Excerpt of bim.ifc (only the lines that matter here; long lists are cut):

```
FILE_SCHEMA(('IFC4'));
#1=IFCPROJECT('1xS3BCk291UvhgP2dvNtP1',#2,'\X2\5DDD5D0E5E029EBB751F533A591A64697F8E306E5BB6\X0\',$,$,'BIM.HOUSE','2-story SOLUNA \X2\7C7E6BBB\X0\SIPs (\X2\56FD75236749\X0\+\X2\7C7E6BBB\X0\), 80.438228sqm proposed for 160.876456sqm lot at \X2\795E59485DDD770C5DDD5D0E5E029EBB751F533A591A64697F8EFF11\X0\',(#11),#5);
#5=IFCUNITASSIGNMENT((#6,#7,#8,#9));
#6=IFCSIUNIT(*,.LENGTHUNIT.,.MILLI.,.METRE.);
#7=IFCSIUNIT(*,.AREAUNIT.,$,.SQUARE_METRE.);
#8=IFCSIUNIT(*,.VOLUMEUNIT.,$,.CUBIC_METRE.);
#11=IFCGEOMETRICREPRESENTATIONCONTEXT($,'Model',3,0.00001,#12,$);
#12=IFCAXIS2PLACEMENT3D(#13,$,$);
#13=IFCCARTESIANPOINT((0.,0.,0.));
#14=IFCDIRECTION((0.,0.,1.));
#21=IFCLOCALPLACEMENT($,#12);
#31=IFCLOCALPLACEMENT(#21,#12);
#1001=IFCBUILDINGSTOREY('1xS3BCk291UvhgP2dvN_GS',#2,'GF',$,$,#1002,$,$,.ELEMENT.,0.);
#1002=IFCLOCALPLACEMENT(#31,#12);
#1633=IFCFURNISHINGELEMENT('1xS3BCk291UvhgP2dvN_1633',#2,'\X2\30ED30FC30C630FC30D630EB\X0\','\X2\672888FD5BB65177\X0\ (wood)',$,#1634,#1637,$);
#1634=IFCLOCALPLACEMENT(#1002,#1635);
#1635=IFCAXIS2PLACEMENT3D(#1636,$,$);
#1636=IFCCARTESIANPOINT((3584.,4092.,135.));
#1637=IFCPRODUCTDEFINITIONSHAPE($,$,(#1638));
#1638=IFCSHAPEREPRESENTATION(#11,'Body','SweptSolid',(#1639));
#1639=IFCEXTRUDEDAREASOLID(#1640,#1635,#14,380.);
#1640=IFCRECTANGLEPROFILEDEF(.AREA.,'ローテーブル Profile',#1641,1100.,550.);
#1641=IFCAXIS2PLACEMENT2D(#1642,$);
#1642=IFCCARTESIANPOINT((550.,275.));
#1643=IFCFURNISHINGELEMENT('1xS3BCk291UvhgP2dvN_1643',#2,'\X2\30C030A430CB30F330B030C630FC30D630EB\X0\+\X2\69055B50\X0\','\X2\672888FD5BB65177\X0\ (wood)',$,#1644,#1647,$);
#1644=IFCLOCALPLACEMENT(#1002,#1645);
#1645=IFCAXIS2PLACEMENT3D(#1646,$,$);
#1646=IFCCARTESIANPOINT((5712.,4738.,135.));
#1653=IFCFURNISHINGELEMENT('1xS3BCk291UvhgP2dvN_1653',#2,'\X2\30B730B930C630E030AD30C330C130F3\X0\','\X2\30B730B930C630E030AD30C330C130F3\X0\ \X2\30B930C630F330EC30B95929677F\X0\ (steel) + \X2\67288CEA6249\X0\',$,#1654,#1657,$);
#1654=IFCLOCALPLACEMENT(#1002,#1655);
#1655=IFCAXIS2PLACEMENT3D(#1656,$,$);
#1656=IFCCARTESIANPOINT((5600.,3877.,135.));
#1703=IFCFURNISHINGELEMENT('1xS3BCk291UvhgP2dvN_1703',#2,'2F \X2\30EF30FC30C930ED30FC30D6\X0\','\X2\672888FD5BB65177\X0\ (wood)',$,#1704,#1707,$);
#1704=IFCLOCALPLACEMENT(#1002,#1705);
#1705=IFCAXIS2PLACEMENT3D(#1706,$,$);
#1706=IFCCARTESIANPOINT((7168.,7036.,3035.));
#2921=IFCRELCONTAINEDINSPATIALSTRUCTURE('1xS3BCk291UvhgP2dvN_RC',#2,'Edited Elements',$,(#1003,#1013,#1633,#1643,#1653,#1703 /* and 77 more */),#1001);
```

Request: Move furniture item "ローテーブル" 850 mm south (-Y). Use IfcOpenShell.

```python
import ifcopenshell
import ifcopenshell.api.geometry
import ifcopenshell.util.placement
import ifcopenshell.util.unit

model = ifcopenshell.open("bim.ifc")
unit_scale = ifcopenshell.util.unit.calculate_unit_scale(model)

item = model.by_id(1633)
matrix = ifcopenshell.util.placement.get_local_placement(item.ObjectPlacement)
matrix[1, 3] -= 0.85 / unit_scale
ifcopenshell.api.geometry.edit_object_placement(model, product=item, matrix=matrix, is_si=False)

print(ifcopenshell.util.placement.get_local_placement(item.ObjectPlacement).round(3) + 0.0)

model.write("bim_updated.ifc")
```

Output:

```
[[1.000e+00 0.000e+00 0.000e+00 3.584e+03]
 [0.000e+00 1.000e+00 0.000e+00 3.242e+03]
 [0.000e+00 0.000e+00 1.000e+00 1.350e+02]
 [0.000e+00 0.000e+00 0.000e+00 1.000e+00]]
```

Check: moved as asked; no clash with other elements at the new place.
